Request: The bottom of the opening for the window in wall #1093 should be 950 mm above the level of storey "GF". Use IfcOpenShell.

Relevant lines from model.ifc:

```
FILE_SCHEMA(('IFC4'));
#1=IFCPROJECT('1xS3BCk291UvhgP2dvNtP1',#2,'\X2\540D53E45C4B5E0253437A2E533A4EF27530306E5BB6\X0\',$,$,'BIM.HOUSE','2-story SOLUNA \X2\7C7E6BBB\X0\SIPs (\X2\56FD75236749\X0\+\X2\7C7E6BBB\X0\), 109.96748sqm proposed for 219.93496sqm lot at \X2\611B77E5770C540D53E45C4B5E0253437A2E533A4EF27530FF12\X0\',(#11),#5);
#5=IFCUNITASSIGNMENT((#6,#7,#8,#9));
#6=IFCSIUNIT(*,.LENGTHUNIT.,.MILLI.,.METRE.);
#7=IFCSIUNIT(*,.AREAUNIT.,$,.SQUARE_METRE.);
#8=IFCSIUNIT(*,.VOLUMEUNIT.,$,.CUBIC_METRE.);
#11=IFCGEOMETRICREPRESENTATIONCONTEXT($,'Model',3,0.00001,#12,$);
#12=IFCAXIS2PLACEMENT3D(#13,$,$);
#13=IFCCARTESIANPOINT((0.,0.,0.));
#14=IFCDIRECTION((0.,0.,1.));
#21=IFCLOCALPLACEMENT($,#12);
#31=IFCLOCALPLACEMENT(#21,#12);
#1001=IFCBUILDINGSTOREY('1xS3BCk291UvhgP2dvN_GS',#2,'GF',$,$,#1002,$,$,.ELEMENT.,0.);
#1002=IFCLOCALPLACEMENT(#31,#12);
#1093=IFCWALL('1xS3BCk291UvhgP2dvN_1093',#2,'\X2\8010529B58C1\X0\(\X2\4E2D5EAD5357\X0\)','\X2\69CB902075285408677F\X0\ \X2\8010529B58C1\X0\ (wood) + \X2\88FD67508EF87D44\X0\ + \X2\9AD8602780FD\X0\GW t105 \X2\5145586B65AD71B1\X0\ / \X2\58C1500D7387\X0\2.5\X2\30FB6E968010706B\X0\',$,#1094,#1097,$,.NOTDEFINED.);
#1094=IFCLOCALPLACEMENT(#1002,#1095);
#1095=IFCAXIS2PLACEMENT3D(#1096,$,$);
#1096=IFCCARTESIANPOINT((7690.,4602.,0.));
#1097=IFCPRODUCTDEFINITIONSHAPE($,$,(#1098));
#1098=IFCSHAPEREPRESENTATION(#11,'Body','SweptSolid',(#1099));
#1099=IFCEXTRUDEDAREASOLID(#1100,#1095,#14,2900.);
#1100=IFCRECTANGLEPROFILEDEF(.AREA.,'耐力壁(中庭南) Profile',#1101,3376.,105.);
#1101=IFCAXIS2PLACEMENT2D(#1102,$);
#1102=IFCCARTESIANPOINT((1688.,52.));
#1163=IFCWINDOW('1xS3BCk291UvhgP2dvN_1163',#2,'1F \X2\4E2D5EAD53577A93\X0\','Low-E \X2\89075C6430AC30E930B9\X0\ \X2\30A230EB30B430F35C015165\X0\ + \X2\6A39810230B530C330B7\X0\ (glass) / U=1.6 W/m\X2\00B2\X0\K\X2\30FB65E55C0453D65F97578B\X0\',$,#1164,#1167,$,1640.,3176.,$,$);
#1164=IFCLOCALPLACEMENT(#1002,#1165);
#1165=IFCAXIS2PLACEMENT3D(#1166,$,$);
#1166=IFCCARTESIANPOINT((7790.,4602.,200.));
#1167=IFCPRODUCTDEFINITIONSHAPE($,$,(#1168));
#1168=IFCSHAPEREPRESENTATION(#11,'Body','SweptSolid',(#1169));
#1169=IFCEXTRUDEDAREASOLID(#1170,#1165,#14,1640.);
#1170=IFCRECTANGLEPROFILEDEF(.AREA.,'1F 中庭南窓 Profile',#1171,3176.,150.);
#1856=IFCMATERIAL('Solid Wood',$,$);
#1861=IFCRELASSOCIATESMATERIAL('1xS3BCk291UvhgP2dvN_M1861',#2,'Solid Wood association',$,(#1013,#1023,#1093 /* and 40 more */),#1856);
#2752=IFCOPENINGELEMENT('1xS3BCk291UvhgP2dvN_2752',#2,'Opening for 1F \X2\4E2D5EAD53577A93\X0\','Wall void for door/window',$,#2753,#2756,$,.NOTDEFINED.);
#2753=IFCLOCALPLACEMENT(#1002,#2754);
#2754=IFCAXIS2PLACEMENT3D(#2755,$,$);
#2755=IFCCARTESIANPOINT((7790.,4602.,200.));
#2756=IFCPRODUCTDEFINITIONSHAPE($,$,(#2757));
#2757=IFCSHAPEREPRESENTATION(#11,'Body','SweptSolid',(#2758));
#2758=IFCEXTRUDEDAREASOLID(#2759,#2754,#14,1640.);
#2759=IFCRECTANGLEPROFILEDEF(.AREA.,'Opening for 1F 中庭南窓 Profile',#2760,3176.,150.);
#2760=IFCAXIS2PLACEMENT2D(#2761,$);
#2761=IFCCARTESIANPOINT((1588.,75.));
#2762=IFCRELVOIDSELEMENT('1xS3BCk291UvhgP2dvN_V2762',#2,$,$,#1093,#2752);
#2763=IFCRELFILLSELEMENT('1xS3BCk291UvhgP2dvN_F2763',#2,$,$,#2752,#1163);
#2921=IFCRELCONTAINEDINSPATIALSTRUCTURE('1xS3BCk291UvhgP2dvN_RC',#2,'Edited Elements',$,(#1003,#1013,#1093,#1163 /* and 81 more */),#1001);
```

```python
import numpy as np
import ifcopenshell
import ifcopenshell.api.geometry
import ifcopenshell.geom
import ifcopenshell.util.element
import ifcopenshell.util.placement
import ifcopenshell.util.shape
import ifcopenshell.util.unit

model = ifcopenshell.open("model.ifc")
unit_scale = ifcopenshell.util.unit.calculate_unit_scale(model)

window = model.by_guid("1xS3BCk291UvhgP2dvN_1163")
opening = window.FillsVoids[0].RelatingOpeningElement
storey = ifcopenshell.util.element.get_container(window, ifc_class="IfcBuildingStorey")
level = ifcopenshell.util.placement.get_local_placement(storey.ObjectPlacement)[2, 3]

# The opening's origin need not be at the sill, so measure its lowest point.
shape = ifcopenshell.geom.create_shape(ifcopenshell.geom.settings(), opening)
bottom = ifcopenshell.util.shape.get_shape_bottom_elevation(shape, shape.geometry) / unit_scale
dz = level + 0.95 / unit_scale - bottom

shift = np.array([0.0, 0.0, dz])
# The window is not placed relative to its opening, so move both.
for product in (opening, window):
    matrix = ifcopenshell.util.placement.get_local_placement(product.ObjectPlacement)
    matrix[:3, 3] += shift
    ifcopenshell.api.geometry.edit_object_placement(model, product=product, matrix=matrix, is_si=False)

print(f"moved by {dz * unit_scale:+.3f} m")

model.write("model-out.ifc")
```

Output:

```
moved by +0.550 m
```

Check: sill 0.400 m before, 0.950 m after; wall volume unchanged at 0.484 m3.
